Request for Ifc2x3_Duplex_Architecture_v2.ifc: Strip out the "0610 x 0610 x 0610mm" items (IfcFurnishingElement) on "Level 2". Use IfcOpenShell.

First a look at what the model holds.

```python
import ifcopenshell
import ifcopenshell.util.element

model = ifcopenshell.open("Ifc2x3_Duplex_Architecture_v2.ifc")
print(model.schema)
storey = next(s for s in model.by_type("IfcBuildingStorey") if s.Name == "Level 2")
furniture = [e for e in ifcopenshell.util.element.get_decomposition(storey) if e.is_a("IfcFurnishingElement")]
seen = {}
for e in furniture:
    element_type = ifcopenshell.util.element.get_type(e)
    name = element_type.Name if element_type not in (None, e) else None
    seen[name] = seen.get(name, 0) + 1
for name, count in sorted(seen.items(), key=str):
    print(count, "x", name)
```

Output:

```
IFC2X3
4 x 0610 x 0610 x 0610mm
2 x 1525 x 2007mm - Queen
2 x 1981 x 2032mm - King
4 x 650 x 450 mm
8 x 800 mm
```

```python
import ifcopenshell
import ifcopenshell.api.root
import ifcopenshell.util.element

model = ifcopenshell.open("Ifc2x3_Duplex_Architecture_v2.ifc")

storey = next(s for s in model.by_type("IfcBuildingStorey") if s.Name == "Level 2")
furniture = [e for e in ifcopenshell.util.element.get_decomposition(storey) if e.is_a("IfcFurnishingElement")]
targets = [e for e in furniture if (t := ifcopenshell.util.element.get_type(e)) not in (None, e) and t.Name == "0610 x 0610 x 0610mm"]

for e in targets:
    ifcopenshell.api.root.remove_product(model, product=e)
print(len(targets), "removed")

model.write("Ifc2x3_Duplex_Architecture_v2-out.ifc")
```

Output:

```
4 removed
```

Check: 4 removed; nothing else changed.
